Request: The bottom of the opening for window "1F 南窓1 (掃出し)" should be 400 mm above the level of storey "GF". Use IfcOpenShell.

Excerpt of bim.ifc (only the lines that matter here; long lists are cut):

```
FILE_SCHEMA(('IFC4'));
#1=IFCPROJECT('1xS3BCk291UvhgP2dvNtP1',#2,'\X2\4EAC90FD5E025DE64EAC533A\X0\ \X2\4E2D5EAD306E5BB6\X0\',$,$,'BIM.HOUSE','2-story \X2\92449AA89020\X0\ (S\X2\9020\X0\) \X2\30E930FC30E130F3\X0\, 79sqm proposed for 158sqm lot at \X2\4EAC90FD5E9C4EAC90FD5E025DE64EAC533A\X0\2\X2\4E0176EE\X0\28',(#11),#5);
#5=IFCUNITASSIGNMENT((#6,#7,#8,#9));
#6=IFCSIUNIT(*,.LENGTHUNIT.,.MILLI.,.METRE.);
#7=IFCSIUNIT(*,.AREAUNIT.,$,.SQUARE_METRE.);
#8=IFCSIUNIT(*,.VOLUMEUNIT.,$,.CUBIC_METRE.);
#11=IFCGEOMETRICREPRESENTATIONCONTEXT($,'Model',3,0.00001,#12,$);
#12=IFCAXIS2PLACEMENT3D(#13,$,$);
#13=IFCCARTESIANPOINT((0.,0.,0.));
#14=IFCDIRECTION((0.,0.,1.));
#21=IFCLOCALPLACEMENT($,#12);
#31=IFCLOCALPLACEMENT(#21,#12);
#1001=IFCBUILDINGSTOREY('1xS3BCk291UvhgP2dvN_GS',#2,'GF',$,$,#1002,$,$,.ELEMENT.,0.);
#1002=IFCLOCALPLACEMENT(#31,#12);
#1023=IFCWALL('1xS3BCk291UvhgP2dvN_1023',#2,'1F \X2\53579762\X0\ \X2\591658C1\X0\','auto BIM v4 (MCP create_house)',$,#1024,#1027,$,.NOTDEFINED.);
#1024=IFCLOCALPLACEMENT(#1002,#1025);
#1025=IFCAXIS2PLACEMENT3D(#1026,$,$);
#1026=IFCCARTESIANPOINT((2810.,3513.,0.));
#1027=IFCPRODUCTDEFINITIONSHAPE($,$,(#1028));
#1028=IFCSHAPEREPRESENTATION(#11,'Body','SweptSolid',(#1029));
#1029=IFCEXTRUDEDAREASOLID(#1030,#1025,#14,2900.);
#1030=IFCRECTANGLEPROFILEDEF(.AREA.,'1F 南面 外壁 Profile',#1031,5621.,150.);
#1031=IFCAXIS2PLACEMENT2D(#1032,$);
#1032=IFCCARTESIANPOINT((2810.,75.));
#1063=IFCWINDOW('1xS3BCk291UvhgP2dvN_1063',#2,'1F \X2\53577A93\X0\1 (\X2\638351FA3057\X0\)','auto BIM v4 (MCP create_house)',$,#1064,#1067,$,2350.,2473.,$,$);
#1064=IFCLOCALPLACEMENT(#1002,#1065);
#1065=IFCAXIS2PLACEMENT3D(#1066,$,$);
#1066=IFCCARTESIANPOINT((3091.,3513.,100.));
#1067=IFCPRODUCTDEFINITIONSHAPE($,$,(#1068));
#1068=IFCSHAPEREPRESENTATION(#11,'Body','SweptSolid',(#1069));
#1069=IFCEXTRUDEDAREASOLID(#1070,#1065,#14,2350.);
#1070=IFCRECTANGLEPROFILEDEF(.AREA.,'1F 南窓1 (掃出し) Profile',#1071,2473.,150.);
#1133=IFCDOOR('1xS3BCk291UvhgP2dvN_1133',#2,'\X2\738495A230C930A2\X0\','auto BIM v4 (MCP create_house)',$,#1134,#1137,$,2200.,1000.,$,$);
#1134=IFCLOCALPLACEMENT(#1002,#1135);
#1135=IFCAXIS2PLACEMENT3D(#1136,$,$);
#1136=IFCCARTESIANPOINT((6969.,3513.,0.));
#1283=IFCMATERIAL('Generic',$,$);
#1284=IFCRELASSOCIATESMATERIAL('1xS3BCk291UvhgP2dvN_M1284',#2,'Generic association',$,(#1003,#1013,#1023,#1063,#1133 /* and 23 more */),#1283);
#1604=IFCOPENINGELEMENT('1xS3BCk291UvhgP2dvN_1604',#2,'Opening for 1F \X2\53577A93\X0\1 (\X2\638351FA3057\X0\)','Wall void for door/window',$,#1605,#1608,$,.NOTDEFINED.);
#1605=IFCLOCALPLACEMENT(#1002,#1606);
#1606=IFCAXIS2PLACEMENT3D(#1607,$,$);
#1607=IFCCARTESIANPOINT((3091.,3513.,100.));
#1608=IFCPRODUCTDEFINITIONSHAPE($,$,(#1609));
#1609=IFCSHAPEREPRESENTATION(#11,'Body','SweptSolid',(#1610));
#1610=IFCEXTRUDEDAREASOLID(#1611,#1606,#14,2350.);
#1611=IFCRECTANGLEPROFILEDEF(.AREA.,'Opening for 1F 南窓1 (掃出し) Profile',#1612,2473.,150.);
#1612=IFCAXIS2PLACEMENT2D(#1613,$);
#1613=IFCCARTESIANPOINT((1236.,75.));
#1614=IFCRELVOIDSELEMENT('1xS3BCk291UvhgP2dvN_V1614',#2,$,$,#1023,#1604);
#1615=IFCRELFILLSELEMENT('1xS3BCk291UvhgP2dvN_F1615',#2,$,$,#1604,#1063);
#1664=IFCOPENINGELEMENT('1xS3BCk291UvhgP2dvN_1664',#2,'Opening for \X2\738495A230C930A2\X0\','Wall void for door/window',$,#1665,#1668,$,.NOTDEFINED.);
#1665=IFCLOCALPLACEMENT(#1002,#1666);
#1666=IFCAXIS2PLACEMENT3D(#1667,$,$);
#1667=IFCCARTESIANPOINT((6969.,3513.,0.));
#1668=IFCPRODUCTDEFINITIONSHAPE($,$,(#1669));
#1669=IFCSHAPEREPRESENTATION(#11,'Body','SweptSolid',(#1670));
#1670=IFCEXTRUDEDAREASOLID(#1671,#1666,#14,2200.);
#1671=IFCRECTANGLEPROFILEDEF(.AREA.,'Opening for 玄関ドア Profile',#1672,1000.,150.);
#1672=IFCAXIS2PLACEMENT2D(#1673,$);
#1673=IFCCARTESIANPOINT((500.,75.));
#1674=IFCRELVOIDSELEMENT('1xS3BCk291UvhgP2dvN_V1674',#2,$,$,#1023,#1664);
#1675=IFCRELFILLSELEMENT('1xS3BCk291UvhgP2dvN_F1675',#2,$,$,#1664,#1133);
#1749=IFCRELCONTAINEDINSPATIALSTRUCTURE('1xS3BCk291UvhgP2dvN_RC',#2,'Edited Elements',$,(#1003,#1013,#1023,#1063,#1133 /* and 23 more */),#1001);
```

```python
import numpy as np
import ifcopenshell
import ifcopenshell.api.geometry
import ifcopenshell.geom
import ifcopenshell.util.element
import ifcopenshell.util.placement
import ifcopenshell.util.shape
import ifcopenshell.util.unit

model = ifcopenshell.open("bim.ifc")
unit_scale = ifcopenshell.util.unit.calculate_unit_scale(model)

window = model.by_id(1063)
opening = window.FillsVoids[0].RelatingOpeningElement
storey = ifcopenshell.util.element.get_container(window, ifc_class="IfcBuildingStorey")
level = ifcopenshell.util.placement.get_local_placement(storey.ObjectPlacement)[2, 3]

# The opening's origin need not be at the sill, so measure its lowest point.
shape = ifcopenshell.geom.create_shape(ifcopenshell.geom.settings(), opening)
bottom = ifcopenshell.util.shape.get_shape_bottom_elevation(shape, shape.geometry) / unit_scale
dz = level + 400.0 - bottom

shift = np.array([0.0, 0.0, dz])
# The window is not placed relative to its opening, so move both.
for product in (opening, window):
    matrix = ifcopenshell.util.placement.get_local_placement(product.ObjectPlacement)
    matrix[:3, 3] += shift
    ifcopenshell.api.geometry.edit_object_placement(model, product=product, matrix=matrix, is_si=False)

print(f"moved by {dz * unit_scale:+.3f} m")

model.write("bim_rev.ifc")
```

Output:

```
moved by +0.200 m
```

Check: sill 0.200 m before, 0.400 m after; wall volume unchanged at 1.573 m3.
